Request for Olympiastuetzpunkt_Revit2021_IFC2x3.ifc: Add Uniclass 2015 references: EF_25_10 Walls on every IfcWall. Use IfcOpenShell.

First a look at what the model holds.

```python
import ifcopenshell

model = ifcopenshell.open("Olympiastuetzpunkt_Revit2021_IFC2x3.ifc")
print(model.schema)
print("classifications:", [c.Name for c in model.by_type("IfcClassification")])
for ifc_class in ("IfcDoor", "IfcRoof", "IfcStair", "IfcWall", "IfcWindow"):
    print(ifc_class, len(model.by_type(ifc_class)))
```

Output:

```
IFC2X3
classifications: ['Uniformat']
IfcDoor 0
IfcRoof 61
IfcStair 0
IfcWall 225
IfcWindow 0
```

```python
import ifcopenshell
import ifcopenshell.api.classification

model = ifcopenshell.open("Olympiastuetzpunkt_Revit2021_IFC2x3.ifc")

# IFC2X3 requires Source and Edition and has no link from the project to the system.
system = model.create_entity("IfcClassification", Source="NBS", Edition="2015", Name="Uniclass 2015")

codes = {
    "IfcWall": ("EF_25_10", "Walls"),
}
for ifc_class, (code, name) in codes.items():
    products = model.by_type(ifc_class)
    ifcopenshell.api.classification.add_reference(
        model, products=products, classification=system, identification=code, name=name
    )
    print(code, len(products))

model.write("Olympiastuetzpunkt_Revit2021_IFC2x3_v2.ifc")
```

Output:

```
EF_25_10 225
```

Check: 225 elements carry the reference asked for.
